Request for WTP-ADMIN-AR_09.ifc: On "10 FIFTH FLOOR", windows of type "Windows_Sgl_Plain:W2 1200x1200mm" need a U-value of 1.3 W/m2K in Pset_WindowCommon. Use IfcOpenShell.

First a look at what the model holds.

```python
import ifcopenshell
import ifcopenshell.util.element

model = ifcopenshell.open("WTP-ADMIN-AR_09.ifc")
print(model.schema)
storey = next(s for s in model.by_type("IfcBuildingStorey") if s.Name == "10 FIFTH FLOOR")
windows = [e for e in ifcopenshell.util.element.get_decomposition(storey) if e.is_a("IfcWindow")]
seen = {}
for e in windows:
    element_type = ifcopenshell.util.element.get_type(e)
    key = (element_type.Name if element_type != e and element_type else None, ifcopenshell.util.element.get_pset(e, "Pset_WindowCommon", "ThermalTransmittance"))
    seen[key] = seen.get(key, 0) + 1
for (name, value), count in sorted(seen.items(), key=str):
    print(count, "x", name, "|", value)
```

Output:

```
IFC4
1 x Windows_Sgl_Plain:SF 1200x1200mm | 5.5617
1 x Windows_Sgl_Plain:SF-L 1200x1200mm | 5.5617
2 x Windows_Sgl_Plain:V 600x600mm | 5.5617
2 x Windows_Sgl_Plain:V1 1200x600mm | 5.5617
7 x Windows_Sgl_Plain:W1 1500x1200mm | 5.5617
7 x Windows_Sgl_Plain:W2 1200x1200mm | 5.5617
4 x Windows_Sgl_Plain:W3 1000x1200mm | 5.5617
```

```python
import ifcopenshell
import ifcopenshell.api.pset
import ifcopenshell.util.element

model = ifcopenshell.open("WTP-ADMIN-AR_09.ifc")

storey = next(s for s in model.by_type("IfcBuildingStorey") if s.Name == "10 FIFTH FLOOR")
windows = [e for e in ifcopenshell.util.element.get_decomposition(storey) if e.is_a("IfcWindow")]

count = 0
for e in windows:
    element_type = ifcopenshell.util.element.get_type(e)
    if element_type in (None, e) or element_type.Name != "Windows_Sgl_Plain:W2 1200x1200mm":
        continue
    # add_pset returns the element's existing set when there is one.
    pset = ifcopenshell.api.pset.add_pset(model, product=e, name="Pset_WindowCommon")
    ifcopenshell.api.pset.edit_pset(model, pset=pset, properties={"ThermalTransmittance": 1.3})
    count += 1

print(count, "windows updated")

model.write("WTP-ADMIN-AR_09_edited.ifc")
```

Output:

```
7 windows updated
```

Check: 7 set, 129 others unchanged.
